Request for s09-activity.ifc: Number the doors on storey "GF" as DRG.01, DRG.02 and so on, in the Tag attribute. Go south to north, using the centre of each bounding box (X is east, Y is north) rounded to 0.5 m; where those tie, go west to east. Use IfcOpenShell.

First a look at what the model holds.

```python
import ifcopenshell
import ifcopenshell.util.element
import ifcopenshell.util.placement

model = ifcopenshell.open("s09-activity.ifc")
print(model.schema)
storey = next(s for s in model.by_type("IfcBuildingStorey") if s.Name == "GF")
doors = [e for e in ifcopenshell.util.element.get_decomposition(storey) if e.is_a("IfcDoor")]
for e in sorted(doors, key=lambda e: e.id()):
    origin = ifcopenshell.util.placement.get_local_placement(e.ObjectPlacement)[:3, 3]
    print(e.id(), e.Tag, e.Name, origin.round(2) + 0.0, sep=" | ")
```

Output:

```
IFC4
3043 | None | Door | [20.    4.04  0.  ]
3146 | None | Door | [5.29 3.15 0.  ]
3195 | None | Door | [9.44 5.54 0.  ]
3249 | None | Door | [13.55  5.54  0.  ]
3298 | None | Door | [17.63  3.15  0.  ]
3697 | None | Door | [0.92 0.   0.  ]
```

```python
import ifcopenshell
import ifcopenshell.geom
import ifcopenshell.util.element
import ifcopenshell.util.shape

model = ifcopenshell.open("s09-activity.ifc")
settings = ifcopenshell.geom.settings()
settings.set("use-world-coords", True)


def centre(element):
    shape = ifcopenshell.geom.create_shape(settings, element)
    return ifcopenshell.util.shape.get_bbox_centroid(shape.geometry)


storey = next(s for s in model.by_type("IfcBuildingStorey") if s.Name == "GF")
doors = [e for e in ifcopenshell.util.element.get_decomposition(storey) if e.is_a("IfcDoor")]

# Insertion points can sit at a corner or the storey origin, so sort by the geometry (in metres).
centres = {e: centre(e) for e in doors}
doors.sort(key=lambda e: (round(centres[e][1] / 0.5), centres[e][0]))

for i, e in enumerate(doors, start=1):
    number = f"DRG.{i:02d}"
    e.Tag = number
    print(e.id(), number)

model.write("s09-activity_edited.ifc")
```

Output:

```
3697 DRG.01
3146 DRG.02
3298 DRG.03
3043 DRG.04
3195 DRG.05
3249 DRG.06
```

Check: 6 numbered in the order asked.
